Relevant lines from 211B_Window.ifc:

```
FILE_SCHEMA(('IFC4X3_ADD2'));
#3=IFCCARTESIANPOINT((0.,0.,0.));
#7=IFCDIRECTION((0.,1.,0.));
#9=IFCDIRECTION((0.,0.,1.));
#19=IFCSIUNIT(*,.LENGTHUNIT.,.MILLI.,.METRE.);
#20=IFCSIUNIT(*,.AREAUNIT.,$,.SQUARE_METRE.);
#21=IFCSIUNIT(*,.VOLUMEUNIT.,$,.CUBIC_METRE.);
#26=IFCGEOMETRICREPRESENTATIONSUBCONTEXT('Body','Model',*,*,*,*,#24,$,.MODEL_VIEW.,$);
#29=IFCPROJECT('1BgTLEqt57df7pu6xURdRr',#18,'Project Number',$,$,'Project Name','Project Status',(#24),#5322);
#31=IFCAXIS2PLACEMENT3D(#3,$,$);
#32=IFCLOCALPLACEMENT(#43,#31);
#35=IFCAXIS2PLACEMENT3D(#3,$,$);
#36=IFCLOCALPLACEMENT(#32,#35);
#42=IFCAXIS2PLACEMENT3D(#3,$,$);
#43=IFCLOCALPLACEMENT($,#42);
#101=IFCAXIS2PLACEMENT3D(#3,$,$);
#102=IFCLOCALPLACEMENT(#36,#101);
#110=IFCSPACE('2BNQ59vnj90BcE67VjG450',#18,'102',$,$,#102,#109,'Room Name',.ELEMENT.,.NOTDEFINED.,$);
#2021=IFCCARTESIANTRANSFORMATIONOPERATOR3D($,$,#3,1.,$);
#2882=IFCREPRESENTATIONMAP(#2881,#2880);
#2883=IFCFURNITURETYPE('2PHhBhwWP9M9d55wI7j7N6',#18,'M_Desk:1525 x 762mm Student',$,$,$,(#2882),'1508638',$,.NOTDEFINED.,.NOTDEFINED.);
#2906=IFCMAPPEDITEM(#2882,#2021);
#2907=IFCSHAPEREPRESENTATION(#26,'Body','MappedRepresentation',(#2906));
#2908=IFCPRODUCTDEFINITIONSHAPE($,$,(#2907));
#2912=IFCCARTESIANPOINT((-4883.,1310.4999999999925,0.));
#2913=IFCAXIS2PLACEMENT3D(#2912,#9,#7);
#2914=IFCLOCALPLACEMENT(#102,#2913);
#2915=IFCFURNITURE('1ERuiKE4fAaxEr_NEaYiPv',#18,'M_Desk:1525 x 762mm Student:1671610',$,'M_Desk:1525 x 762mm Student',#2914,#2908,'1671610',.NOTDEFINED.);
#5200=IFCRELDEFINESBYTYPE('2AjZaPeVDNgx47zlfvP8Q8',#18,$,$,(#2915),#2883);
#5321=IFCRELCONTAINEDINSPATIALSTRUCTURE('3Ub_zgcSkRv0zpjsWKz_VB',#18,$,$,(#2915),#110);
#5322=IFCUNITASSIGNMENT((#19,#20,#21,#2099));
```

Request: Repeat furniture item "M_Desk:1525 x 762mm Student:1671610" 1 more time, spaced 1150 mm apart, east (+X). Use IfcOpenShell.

```python
import numpy as np
import ifcopenshell
import ifcopenshell.api.geometry
import ifcopenshell.api.root
import ifcopenshell.util.element
import ifcopenshell.util.placement

model = ifcopenshell.open("211B_Window.ifc")


def reuse_history(source, copy):
    """copy_class also copies each property set's owner history, people and application; keep the originals."""
    for rel in copy.IsDefinedBy:
        if rel.is_a("IfcRelDefinesByProperties") and (history := rel.RelatingPropertyDefinition.OwnerHistory):
            rel.RelatingPropertyDefinition.OwnerHistory = source.OwnerHistory
            ifcopenshell.util.element.remove_deep2(model, history)


source = model.by_guid("1ERuiKE4fAaxEr_NEaYiPv")
base = ifcopenshell.util.placement.get_local_placement(source.ObjectPlacement)
step = np.array([1.0, 0.0, 0.0]) * 1150.0

for i in range(1, 2):
    copy = ifcopenshell.api.root.copy_class(model, product=source)
    copy.Representation = ifcopenshell.util.element.copy_deep(
        model, source.Representation, exclude=["IfcGeometricRepresentationContext", "IfcRepresentationMap"]
    )
    copy.Name = "M_Desk:1525 x 762mm Student"
    copy.Tag = None
    reuse_history(source, copy)
    matrix = base.copy()
    matrix[:3, 3] += i * step
    print("added at", matrix[:3, 3].round(3) + 0.0)
    ifcopenshell.api.geometry.edit_object_placement(model, product=copy, matrix=matrix, is_si=False)

model.write("211B_Window_v2.ifc")
```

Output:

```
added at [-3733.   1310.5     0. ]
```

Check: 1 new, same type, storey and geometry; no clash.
